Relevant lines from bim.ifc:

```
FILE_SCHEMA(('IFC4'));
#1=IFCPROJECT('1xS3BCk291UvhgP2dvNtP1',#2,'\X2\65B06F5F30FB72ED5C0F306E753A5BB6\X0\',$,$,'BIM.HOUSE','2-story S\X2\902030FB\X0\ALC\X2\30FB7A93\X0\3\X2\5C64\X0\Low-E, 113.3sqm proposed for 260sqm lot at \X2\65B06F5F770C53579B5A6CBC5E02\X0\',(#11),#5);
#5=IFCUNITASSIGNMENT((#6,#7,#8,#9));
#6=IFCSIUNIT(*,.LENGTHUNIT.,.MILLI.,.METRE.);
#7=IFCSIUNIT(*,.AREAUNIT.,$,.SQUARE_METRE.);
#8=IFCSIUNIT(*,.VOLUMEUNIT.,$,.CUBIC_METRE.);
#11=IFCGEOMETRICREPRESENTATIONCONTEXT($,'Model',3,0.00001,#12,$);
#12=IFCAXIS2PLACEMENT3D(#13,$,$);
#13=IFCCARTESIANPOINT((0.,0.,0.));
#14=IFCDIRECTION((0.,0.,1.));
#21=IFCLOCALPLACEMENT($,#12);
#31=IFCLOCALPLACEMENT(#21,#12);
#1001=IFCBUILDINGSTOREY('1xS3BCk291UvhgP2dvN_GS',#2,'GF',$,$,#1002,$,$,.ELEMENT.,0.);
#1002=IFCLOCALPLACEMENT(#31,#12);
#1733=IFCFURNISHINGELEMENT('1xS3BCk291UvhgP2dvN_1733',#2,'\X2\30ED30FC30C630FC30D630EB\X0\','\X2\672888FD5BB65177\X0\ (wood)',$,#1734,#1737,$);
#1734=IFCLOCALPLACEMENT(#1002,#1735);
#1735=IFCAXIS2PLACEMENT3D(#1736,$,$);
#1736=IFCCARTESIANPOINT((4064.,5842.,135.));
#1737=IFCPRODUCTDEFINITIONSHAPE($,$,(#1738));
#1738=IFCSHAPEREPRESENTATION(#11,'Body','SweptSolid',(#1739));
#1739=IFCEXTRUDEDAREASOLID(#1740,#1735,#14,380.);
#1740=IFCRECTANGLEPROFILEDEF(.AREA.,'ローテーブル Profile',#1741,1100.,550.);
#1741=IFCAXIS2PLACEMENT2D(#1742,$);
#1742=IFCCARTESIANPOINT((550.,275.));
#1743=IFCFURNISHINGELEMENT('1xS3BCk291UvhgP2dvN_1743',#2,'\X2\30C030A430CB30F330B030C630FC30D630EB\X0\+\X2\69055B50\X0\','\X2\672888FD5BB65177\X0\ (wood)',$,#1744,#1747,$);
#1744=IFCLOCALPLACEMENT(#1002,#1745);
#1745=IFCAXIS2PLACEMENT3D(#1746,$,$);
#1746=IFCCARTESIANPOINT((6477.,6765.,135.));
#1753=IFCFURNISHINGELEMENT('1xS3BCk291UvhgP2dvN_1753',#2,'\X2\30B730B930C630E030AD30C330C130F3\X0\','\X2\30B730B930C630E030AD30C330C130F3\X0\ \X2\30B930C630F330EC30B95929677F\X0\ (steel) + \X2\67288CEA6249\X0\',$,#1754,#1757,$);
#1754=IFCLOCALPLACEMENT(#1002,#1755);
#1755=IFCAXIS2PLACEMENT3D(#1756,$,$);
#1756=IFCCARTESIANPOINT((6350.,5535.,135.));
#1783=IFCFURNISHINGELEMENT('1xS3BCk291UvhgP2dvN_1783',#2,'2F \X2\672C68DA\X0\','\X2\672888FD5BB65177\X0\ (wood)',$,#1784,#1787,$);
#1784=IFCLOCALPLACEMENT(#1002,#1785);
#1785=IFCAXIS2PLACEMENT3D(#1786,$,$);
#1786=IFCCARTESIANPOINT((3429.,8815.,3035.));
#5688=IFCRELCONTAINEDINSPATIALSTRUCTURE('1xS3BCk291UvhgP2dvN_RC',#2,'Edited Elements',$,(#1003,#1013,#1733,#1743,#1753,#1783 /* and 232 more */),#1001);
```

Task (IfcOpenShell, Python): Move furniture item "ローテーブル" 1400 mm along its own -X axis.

```python
import ifcopenshell
import ifcopenshell.api.geometry
import ifcopenshell.util.placement
import ifcopenshell.util.unit

model = ifcopenshell.open("bim.ifc")
unit_scale = ifcopenshell.util.unit.calculate_unit_scale(model)

item = model.by_guid("1xS3BCk291UvhgP2dvN_1733")
matrix = ifcopenshell.util.placement.get_local_placement(item.ObjectPlacement)
matrix[:3, 3] -= matrix[:3, 0] * 1.4 / unit_scale
ifcopenshell.api.geometry.edit_object_placement(model, product=item, matrix=matrix, is_si=False)

print(ifcopenshell.util.placement.get_local_placement(item.ObjectPlacement).round(3) + 0.0)

model.write("bim_edited.ifc")
```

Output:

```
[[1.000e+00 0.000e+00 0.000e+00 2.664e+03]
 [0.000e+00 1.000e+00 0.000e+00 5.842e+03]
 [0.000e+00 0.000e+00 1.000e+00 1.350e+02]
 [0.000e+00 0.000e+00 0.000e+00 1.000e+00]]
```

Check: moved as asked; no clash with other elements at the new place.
